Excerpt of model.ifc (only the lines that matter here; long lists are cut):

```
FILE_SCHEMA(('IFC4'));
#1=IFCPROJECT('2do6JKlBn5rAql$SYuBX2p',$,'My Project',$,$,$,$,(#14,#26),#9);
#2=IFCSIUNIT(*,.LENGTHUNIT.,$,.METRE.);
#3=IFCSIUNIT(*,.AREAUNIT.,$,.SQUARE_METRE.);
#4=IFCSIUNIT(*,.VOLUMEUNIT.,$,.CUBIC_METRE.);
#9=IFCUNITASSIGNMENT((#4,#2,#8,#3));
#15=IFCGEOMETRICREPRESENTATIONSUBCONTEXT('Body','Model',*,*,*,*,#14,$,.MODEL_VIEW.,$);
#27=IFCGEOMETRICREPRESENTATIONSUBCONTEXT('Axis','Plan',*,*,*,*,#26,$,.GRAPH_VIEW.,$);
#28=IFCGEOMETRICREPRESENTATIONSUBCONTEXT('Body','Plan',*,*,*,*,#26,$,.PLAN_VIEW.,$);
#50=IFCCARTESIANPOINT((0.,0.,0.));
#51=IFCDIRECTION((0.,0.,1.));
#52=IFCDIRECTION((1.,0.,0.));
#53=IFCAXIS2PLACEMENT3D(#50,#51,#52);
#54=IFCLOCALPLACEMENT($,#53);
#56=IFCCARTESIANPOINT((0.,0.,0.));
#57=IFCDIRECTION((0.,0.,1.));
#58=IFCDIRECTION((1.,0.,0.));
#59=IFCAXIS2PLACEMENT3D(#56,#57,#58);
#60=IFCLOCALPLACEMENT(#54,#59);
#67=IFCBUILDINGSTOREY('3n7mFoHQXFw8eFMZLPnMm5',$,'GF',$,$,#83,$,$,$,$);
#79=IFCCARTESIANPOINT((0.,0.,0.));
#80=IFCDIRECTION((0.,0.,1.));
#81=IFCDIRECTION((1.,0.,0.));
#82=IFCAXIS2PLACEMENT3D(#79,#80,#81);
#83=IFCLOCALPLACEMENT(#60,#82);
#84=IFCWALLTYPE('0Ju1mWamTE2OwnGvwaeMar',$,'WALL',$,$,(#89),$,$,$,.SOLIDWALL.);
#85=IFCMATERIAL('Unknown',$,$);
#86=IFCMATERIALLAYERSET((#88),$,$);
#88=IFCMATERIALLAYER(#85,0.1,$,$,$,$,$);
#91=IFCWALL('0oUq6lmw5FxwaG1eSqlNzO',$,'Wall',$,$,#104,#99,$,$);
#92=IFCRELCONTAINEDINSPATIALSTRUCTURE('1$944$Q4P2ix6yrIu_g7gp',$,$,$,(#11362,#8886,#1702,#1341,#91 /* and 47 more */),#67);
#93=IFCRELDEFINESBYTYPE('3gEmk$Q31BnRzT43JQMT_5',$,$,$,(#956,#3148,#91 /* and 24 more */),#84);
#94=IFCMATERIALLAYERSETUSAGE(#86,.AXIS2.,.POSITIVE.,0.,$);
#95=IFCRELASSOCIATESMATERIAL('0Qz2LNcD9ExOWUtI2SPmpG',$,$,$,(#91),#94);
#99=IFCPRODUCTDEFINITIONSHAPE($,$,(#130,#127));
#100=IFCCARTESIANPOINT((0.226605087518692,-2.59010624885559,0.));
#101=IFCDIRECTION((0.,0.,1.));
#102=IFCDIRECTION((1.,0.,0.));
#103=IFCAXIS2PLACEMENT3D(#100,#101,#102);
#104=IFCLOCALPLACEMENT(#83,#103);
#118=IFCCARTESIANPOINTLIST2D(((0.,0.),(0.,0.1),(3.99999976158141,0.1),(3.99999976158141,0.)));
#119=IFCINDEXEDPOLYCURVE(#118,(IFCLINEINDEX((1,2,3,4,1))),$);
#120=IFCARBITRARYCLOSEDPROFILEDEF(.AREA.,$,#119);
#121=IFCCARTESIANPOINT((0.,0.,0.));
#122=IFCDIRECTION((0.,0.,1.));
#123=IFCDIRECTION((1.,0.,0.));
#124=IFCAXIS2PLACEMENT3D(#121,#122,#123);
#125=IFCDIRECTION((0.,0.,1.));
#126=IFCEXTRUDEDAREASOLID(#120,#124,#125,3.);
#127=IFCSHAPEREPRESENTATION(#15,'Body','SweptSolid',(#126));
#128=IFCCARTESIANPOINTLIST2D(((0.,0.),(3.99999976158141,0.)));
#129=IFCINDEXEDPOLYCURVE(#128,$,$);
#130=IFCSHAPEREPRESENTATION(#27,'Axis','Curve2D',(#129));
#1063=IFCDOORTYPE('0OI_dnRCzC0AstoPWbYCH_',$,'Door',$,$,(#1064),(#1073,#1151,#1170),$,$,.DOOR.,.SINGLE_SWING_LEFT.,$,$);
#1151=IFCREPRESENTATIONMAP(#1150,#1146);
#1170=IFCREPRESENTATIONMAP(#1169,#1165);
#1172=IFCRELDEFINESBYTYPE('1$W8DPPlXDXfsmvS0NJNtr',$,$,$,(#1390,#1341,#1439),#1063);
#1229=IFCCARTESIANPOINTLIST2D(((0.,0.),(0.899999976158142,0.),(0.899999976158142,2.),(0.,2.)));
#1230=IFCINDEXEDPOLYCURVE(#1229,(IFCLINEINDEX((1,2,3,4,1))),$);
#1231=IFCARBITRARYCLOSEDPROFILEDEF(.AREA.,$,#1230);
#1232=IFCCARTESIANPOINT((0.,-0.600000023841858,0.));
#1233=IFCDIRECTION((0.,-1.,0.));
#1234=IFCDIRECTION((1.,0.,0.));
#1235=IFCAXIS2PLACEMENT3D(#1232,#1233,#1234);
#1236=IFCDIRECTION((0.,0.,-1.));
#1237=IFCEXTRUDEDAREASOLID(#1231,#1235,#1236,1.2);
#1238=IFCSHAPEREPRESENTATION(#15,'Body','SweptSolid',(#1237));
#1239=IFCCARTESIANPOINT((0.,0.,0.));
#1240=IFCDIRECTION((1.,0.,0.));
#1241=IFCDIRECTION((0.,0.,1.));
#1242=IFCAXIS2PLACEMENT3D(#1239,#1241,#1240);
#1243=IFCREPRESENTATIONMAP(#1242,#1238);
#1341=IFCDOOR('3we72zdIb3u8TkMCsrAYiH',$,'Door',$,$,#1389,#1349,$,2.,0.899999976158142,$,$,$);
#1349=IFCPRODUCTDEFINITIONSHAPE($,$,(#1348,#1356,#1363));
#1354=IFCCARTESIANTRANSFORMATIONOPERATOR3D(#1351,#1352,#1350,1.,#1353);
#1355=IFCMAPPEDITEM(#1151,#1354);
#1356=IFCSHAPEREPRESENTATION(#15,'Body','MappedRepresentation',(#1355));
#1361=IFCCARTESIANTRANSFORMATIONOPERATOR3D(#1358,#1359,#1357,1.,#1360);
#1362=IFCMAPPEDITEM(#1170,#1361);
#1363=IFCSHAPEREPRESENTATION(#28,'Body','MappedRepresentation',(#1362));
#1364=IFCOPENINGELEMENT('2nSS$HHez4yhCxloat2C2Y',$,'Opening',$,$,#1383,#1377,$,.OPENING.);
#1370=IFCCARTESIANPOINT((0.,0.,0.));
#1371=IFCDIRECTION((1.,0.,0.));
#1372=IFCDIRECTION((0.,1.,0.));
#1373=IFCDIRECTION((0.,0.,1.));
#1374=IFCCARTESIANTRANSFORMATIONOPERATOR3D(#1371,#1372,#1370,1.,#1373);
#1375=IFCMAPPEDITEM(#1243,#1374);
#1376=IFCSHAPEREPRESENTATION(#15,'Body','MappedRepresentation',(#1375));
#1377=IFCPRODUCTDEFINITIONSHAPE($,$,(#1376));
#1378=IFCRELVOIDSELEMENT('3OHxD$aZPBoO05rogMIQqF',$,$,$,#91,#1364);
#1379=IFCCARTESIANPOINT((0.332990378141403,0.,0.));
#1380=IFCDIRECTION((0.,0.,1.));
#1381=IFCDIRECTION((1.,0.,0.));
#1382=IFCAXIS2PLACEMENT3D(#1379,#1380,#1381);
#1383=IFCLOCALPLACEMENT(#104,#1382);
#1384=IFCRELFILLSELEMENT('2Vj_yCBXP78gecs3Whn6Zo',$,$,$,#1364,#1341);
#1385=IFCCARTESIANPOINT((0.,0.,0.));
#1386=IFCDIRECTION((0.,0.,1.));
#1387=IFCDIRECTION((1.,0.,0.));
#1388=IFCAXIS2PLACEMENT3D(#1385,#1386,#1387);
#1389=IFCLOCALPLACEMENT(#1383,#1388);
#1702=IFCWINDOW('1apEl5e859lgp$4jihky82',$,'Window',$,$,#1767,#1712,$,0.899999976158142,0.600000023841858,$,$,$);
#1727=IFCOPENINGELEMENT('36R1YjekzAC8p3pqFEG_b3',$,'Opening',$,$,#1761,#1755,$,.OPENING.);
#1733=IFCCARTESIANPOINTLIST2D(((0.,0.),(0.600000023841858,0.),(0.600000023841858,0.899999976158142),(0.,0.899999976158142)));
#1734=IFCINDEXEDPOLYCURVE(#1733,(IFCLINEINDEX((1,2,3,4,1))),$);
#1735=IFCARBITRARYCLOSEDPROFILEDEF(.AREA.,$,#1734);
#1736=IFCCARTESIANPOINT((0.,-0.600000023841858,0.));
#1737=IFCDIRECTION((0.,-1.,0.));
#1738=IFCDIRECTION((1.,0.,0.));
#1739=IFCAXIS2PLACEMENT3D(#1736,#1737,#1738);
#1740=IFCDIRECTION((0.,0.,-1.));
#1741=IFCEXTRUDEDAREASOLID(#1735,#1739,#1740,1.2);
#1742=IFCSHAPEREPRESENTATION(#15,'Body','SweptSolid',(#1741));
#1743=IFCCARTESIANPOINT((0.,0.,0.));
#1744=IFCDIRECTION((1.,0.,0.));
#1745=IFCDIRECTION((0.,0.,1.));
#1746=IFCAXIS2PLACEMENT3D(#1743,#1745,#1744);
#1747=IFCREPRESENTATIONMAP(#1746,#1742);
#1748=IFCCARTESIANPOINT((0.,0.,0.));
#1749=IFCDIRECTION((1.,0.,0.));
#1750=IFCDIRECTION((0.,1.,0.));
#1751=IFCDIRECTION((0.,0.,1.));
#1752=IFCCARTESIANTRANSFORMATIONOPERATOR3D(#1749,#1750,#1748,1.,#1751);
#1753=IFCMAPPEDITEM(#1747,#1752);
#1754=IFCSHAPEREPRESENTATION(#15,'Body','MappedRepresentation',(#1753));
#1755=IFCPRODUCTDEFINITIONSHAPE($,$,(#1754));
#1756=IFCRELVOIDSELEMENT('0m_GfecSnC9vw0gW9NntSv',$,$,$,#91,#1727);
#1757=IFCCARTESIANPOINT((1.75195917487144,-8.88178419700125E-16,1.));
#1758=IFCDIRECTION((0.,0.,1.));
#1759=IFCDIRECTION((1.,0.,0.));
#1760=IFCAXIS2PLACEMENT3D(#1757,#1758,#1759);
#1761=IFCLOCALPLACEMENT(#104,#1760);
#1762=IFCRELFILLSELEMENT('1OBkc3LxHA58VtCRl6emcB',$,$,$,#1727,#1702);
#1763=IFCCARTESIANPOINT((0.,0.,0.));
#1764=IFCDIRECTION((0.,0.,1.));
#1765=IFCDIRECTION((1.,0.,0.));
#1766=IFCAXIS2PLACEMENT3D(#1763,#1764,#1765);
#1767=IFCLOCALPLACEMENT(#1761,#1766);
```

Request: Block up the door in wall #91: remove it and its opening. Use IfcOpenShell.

```python
import ifcopenshell
import ifcopenshell.api.feature
import ifcopenshell.api.root
import ifcopenshell.geom
import ifcopenshell.util.shape

model = ifcopenshell.open("model.ifc")
settings = ifcopenshell.geom.settings()


def volume(element):
    """Net volume in cubic metres, openings subtracted."""
    shape = ifcopenshell.geom.create_shape(settings, element)
    return ifcopenshell.util.shape.get_volume(shape.geometry)


door = model.by_guid("3we72zdIb3u8TkMCsrAYiH")
opening = door.FillsVoids[0].RelatingOpeningElement
wall = opening.VoidsElements[0].RelatingBuildingElement
before = volume(wall)

ifcopenshell.api.root.remove_product(model, product=door)
ifcopenshell.api.feature.remove_feature(model, feature=opening)

after = volume(wall)

print(f"wall volume {before:.3f} -> {after:.3f} m3")

model.write("model_v2.ifc")
```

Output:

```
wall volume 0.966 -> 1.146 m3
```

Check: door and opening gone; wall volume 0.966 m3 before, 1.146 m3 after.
